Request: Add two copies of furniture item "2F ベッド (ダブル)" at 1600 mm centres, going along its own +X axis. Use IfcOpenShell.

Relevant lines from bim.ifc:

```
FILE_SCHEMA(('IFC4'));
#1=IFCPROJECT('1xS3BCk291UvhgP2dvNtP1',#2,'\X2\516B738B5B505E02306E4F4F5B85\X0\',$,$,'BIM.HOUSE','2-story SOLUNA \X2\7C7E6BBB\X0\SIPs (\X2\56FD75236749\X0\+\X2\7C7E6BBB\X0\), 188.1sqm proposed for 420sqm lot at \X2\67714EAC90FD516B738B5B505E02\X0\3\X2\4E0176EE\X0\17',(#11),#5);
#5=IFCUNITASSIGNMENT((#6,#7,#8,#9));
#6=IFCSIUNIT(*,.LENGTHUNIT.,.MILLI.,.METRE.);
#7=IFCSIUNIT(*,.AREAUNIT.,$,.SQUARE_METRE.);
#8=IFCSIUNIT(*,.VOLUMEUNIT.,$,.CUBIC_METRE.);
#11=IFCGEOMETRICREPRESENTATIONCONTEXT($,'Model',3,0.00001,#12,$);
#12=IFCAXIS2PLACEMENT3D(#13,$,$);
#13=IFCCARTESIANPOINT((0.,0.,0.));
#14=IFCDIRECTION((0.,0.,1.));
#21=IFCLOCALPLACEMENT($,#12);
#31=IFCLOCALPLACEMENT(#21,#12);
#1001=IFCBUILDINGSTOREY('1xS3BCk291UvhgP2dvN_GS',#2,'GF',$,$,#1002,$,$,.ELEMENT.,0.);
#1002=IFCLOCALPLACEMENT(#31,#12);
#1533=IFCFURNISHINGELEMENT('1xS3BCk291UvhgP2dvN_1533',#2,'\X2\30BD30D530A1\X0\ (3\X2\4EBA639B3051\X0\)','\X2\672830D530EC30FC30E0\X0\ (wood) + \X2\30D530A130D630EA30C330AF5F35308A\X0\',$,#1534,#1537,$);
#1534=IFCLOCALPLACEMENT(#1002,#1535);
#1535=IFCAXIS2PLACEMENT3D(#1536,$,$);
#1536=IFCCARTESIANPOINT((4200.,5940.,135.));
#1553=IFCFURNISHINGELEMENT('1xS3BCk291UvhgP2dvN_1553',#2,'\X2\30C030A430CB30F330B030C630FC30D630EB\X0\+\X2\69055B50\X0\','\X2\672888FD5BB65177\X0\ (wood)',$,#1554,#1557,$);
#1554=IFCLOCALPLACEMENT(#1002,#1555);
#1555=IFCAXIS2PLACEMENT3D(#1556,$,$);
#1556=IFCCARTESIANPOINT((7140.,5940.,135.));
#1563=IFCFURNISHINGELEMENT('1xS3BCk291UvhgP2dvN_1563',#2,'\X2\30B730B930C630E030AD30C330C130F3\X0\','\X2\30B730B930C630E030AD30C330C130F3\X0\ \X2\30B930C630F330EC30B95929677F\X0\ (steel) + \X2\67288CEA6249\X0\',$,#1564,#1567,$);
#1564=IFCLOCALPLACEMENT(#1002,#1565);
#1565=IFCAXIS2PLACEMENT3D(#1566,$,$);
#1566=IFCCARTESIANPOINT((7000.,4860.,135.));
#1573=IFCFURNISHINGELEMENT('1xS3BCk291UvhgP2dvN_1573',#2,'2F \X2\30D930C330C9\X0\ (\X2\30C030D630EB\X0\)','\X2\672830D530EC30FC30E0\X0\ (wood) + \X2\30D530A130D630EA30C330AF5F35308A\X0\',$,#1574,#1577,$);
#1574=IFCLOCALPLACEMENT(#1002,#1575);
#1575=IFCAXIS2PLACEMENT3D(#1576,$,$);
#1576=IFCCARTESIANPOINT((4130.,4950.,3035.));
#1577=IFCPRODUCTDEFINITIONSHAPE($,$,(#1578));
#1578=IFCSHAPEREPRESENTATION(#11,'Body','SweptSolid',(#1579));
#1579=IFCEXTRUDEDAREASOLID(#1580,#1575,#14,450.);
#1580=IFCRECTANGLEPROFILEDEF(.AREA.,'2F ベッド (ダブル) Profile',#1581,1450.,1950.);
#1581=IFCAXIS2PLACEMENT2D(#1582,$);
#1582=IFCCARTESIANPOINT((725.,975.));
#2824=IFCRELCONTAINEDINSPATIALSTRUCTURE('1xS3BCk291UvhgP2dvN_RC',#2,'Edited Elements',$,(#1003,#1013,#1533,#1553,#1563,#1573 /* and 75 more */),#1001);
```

```python
import ifcopenshell
import ifcopenshell.api.geometry
import ifcopenshell.api.root
import ifcopenshell.util.element
import ifcopenshell.util.placement

model = ifcopenshell.open("bim.ifc")


def reuse_history(source, copy):
    """copy_class also copies each property set's owner history, people and application; keep the originals."""
    for rel in copy.IsDefinedBy:
        if rel.is_a("IfcRelDefinesByProperties") and (history := rel.RelatingPropertyDefinition.OwnerHistory):
            rel.RelatingPropertyDefinition.OwnerHistory = source.OwnerHistory
            ifcopenshell.util.element.remove_deep2(model, history)


source = model.by_id(1573)
base = ifcopenshell.util.placement.get_local_placement(source.ObjectPlacement)
step = base[:3, 0] * 1600.0

for i in range(1, 3):
    copy = ifcopenshell.api.root.copy_class(model, product=source)
    copy.Representation = ifcopenshell.util.element.copy_deep(
        model, source.Representation, exclude=["IfcGeometricRepresentationContext", "IfcRepresentationMap"]
    )
    reuse_history(source, copy)
    matrix = base.copy()
    matrix[:3, 3] += i * step
    print("added at", matrix[:3, 3].round(3) + 0.0)
    ifcopenshell.api.geometry.edit_object_placement(model, product=copy, matrix=matrix, is_si=False)

model.write("bim_edited.ifc")
```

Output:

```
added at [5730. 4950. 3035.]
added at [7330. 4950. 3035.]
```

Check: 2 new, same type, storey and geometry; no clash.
